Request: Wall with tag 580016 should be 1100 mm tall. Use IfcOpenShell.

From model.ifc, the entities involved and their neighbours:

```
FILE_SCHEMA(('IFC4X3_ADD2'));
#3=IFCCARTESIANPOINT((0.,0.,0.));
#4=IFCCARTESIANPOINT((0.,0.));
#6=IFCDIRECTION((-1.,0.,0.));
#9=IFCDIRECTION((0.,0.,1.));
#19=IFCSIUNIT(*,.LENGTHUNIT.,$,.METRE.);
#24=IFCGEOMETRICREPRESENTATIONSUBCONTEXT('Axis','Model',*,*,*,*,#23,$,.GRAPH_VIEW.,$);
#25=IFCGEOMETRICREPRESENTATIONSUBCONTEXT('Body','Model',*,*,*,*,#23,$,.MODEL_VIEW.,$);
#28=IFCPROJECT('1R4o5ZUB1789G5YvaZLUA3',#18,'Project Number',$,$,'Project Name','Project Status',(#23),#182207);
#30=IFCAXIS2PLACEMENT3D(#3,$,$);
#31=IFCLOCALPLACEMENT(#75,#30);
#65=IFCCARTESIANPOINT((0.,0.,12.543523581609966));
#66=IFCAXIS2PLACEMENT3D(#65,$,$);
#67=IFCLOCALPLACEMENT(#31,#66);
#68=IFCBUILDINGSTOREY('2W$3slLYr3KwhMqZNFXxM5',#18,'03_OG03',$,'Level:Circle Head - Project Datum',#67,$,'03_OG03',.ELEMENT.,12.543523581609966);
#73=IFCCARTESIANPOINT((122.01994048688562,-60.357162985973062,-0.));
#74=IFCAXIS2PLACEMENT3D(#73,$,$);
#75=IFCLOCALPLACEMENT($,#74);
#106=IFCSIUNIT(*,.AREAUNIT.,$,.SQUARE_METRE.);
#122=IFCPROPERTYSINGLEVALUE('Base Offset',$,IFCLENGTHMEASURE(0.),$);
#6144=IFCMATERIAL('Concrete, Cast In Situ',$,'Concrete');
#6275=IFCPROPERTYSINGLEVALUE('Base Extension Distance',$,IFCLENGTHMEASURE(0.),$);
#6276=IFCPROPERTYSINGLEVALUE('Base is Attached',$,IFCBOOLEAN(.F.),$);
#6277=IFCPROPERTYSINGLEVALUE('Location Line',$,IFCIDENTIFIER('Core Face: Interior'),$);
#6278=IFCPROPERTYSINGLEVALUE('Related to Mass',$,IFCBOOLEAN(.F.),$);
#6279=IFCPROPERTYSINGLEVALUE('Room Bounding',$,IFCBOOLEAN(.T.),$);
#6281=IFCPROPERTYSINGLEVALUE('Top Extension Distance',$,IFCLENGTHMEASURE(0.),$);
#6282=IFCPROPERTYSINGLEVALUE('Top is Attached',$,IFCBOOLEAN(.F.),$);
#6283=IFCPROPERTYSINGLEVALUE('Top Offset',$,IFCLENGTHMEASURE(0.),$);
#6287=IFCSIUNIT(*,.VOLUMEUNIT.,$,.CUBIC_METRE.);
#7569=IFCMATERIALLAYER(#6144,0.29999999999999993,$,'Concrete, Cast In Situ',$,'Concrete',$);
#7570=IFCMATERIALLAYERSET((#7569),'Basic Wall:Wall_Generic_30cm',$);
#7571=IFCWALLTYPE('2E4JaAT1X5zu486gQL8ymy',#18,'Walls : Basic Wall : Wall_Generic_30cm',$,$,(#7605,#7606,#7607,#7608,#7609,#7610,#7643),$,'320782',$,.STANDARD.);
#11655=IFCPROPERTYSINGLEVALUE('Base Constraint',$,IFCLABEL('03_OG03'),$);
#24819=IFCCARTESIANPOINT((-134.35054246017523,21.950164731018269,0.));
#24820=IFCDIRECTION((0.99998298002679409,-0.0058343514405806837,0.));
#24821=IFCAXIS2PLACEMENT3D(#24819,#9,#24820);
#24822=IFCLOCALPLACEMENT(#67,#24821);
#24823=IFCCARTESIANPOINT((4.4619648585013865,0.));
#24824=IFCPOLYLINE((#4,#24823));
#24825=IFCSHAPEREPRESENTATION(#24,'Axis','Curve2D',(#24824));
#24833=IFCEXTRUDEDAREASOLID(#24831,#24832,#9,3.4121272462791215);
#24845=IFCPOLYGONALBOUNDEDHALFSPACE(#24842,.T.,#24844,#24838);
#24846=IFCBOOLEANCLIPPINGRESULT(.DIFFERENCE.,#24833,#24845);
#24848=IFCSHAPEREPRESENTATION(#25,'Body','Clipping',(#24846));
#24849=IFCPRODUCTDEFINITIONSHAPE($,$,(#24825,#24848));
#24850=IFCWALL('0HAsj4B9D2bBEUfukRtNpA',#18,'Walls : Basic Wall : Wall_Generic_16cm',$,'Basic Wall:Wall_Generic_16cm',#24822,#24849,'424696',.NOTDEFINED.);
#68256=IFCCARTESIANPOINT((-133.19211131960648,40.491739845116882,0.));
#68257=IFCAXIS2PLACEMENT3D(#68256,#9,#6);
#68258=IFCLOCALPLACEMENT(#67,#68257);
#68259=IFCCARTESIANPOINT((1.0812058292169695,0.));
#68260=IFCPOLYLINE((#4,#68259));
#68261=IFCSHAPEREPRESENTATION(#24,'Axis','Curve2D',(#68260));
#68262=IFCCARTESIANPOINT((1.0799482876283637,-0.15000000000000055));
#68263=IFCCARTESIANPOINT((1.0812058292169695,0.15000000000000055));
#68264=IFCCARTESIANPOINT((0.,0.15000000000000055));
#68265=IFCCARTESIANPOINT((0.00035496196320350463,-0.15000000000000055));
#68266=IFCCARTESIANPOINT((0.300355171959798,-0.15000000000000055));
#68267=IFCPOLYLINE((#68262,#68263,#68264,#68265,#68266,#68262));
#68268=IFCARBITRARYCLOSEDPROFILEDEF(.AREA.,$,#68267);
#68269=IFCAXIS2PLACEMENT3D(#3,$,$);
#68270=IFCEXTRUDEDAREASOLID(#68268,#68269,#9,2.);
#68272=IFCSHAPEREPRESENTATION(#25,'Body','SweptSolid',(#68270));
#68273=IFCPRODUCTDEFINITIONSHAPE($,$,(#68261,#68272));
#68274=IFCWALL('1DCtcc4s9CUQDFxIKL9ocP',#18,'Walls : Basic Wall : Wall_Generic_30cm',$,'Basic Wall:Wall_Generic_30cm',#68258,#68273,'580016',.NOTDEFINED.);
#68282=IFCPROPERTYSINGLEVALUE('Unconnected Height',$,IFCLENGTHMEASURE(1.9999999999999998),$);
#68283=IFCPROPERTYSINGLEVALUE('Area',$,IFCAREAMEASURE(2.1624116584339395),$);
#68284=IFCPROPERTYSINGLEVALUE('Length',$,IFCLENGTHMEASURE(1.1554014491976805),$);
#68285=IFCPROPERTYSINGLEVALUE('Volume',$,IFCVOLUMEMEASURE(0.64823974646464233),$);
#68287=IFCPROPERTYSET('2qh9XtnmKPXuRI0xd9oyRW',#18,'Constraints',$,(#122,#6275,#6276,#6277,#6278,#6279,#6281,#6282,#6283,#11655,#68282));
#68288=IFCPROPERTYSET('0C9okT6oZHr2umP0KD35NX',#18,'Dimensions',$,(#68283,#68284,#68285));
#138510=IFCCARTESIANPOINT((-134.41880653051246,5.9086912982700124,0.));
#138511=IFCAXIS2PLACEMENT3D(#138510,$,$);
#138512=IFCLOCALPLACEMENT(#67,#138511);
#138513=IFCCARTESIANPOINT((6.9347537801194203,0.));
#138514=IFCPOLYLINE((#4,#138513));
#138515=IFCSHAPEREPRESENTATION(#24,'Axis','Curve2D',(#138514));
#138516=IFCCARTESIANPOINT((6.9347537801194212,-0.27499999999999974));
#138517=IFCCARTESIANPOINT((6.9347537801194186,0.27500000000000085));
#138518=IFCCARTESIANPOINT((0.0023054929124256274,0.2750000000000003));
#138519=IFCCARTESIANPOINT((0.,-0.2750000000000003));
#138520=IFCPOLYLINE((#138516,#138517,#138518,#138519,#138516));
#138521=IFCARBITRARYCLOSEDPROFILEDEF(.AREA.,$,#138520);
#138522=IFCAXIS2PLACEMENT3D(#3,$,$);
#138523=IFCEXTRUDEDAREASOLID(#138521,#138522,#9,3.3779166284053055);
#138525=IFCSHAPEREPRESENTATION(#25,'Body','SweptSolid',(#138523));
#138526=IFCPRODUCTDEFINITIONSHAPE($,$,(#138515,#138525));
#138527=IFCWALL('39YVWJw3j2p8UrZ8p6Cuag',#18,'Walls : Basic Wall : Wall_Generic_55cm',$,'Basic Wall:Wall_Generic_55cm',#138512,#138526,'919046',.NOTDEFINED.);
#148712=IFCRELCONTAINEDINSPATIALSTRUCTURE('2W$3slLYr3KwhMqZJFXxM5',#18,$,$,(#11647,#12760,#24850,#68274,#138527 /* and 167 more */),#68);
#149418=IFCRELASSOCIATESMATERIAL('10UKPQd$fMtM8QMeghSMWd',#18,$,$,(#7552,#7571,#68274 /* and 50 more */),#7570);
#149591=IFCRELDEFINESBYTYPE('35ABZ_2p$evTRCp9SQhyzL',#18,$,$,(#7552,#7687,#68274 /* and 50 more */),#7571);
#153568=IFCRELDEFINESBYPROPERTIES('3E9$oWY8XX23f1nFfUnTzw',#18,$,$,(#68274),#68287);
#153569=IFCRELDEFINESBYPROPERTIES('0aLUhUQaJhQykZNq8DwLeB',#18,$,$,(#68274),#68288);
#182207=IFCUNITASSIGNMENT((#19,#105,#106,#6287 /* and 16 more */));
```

```python
import ifcopenshell
import ifcopenshell.api.pset
import ifcopenshell.geom
import ifcopenshell.util.element
import ifcopenshell.util.representation
import ifcopenshell.util.shape
import ifcopenshell.util.unit

model = ifcopenshell.open("model.ifc")
unit_scale = ifcopenshell.util.unit.calculate_unit_scale(model)
area_scale = ifcopenshell.util.unit.calculate_unit_scale(model, "AREAUNIT")
volume_scale = ifcopenshell.util.unit.calculate_unit_scale(model, "VOLUMEUNIT")
settings = ifcopenshell.geom.settings()


def volume(element):
    """Net volume in cubic metres, openings subtracted."""
    shape = ifcopenshell.geom.create_shape(settings, element)
    return ifcopenshell.util.shape.get_volume(shape.geometry)


wall = model.by_guid("1DCtcc4s9CUQDFxIKL9ocP")
before = volume(wall)

body = ifcopenshell.util.representation.get_representation(wall, "Model", "Body")
solid = body.Items[0]
old_height = solid.Depth
solid.Depth = 1.1 / unit_scale
after = volume(wall)
thickness = 0.3  # wall thickness in metres

# Update the stored height, areas and volumes.
pset = model.by_id(ifcopenshell.util.element.get_pset(wall, "Constraints", should_inherit=False)["id"])
ifcopenshell.api.pset.edit_pset(model, pset=pset, properties={
    "Unconnected Height": model.create_entity("IfcLengthMeasure", solid.Depth),
})
pset = model.by_id(ifcopenshell.util.element.get_pset(wall, "Dimensions", should_inherit=False)["id"])
ifcopenshell.api.pset.edit_pset(model, pset=pset, properties={
    "Area": model.create_entity("IfcAreaMeasure", after / thickness / area_scale),
    "Volume": model.create_entity("IfcVolumeMeasure", after / volume_scale),
})

print(f"height {old_height:g} -> {solid.Depth:g}, volume {before:.3f} -> {after:.3f} m3")

model.write("model_rev.ifc")
```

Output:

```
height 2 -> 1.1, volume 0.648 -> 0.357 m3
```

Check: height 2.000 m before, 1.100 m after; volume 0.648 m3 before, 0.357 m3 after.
